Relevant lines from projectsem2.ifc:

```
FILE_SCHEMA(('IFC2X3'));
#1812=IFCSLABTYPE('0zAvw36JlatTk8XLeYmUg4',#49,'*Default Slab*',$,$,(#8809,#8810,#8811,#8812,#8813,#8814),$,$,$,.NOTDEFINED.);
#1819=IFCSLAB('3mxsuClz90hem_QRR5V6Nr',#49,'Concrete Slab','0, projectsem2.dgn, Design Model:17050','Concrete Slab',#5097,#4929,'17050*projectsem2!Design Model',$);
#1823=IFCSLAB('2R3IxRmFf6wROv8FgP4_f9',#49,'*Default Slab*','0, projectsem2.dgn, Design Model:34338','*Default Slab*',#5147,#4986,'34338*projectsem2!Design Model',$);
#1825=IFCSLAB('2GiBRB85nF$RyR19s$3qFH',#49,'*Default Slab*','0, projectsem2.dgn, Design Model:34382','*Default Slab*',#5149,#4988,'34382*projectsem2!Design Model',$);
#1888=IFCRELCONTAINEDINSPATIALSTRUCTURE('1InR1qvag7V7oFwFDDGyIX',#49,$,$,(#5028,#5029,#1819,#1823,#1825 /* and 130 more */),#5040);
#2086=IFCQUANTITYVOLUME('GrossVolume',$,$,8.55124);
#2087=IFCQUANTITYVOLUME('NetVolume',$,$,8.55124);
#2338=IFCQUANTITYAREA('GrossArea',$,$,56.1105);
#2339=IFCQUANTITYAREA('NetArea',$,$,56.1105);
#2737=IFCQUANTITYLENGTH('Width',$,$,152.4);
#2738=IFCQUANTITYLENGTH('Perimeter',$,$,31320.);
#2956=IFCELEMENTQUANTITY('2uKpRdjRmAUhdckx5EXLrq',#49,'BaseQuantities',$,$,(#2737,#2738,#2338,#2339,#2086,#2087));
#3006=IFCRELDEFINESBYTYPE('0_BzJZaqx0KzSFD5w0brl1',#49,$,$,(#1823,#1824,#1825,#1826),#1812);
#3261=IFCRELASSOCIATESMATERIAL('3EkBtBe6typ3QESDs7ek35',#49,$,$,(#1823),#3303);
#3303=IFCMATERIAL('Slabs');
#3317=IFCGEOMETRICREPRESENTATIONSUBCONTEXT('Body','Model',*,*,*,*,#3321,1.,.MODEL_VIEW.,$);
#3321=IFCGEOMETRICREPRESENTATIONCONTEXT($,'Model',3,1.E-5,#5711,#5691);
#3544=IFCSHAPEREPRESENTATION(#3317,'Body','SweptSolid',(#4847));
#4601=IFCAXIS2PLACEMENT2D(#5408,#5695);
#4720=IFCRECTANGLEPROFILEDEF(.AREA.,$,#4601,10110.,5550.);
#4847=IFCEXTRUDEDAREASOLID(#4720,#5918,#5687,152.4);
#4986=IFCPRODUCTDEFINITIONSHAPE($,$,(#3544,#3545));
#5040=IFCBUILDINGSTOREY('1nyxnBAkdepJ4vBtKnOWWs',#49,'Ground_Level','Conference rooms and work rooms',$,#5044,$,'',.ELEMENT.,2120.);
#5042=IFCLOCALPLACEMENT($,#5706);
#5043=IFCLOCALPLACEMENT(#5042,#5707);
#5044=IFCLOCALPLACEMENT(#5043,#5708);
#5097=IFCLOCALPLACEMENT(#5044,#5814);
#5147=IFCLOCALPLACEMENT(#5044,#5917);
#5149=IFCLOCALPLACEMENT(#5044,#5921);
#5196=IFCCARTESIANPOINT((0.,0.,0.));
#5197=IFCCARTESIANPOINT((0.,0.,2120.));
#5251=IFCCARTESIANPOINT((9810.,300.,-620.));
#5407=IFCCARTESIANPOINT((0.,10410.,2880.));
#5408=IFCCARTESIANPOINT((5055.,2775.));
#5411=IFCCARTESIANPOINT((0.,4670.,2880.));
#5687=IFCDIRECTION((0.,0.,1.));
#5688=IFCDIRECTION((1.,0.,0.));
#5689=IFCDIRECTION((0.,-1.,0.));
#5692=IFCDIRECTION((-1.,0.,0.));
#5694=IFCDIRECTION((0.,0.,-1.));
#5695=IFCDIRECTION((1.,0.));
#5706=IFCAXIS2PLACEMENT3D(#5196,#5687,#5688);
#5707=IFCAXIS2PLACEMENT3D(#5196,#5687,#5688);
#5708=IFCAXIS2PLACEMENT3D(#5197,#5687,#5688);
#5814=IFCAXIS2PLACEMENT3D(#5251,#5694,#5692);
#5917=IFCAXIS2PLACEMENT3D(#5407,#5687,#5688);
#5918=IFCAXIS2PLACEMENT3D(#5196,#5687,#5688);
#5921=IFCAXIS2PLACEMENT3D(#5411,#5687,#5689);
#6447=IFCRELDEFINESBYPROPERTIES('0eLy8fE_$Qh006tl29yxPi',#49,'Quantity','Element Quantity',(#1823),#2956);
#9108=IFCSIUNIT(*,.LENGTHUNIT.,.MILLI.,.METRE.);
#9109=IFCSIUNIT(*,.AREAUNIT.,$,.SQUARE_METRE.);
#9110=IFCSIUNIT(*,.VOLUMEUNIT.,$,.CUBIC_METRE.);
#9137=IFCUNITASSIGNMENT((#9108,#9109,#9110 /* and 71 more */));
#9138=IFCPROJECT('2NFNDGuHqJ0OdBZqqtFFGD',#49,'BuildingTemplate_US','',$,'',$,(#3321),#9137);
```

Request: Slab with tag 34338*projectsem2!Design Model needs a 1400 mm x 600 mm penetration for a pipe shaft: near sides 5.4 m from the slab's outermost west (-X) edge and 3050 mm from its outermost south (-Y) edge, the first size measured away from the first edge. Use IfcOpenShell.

```python
import numpy as np
import ifcopenshell
import ifcopenshell.api.feature
import ifcopenshell.api.geometry
import ifcopenshell.api.pset
import ifcopenshell.api.root
import ifcopenshell.geom
import ifcopenshell.util.element
import ifcopenshell.util.placement
import ifcopenshell.util.representation
import ifcopenshell.util.shape
import ifcopenshell.util.unit

model = ifcopenshell.open("projectsem2.ifc")
unit_scale = ifcopenshell.util.unit.calculate_unit_scale(model)
area_scale = ifcopenshell.util.unit.calculate_unit_scale(model, "AREAUNIT")
volume_scale = ifcopenshell.util.unit.calculate_unit_scale(model, "VOLUMEUNIT")
settings = ifcopenshell.geom.settings()


def volume(element):
    """Net volume in cubic metres, openings subtracted."""
    shape = ifcopenshell.geom.create_shape(settings, element)
    return ifcopenshell.util.shape.get_volume(shape.geometry)


slab = model.by_id(1823)
before = volume(slab)

# Extent in the slab's own axes, in metres. The edges named are its -X and -Y sides.
slab_shape = ifcopenshell.geom.create_shape(settings, slab)
vertices = ifcopenshell.util.shape.get_vertices(slab_shape.geometry)
x_min, y_min, bottom = vertices.min(axis=0)
top = vertices[:, 2].max()

opening = ifcopenshell.api.root.create_entity(model, ifc_class="IfcOpeningElement", name="Pipe shaft opening")
context = ifcopenshell.util.representation.get_context(model, "Model", "Body", "MODEL_VIEW")
width, depth = 1.4, 0.6
outline = [(0.0, 0.0), (width, 0.0), (width, depth), (0.0, depth), (0.0, 0.0)]
# Overshoot both faces by 50 mm so the cut is clean.
shape = ifcopenshell.api.geometry.add_slab_representation(
    model, context=context, depth=top - bottom + 0.1, polyline=outline
)
ifcopenshell.api.geometry.assign_representation(model, product=opening, representation=shape)

matrix = ifcopenshell.util.placement.get_local_placement(slab.ObjectPlacement)
matrix[:, 3] = matrix @ np.append(np.array([x_min + 5.4, y_min + 3.05, bottom - 0.05]) / unit_scale, 1.0)
ifcopenshell.api.geometry.edit_object_placement(model, product=opening, matrix=matrix, is_si=False)
ifcopenshell.api.feature.add_feature(model, feature=opening, element=slab)

after = volume(slab)

# Update the slab's stored quantities.
qto = model.by_id(ifcopenshell.util.element.get_pset(slab, "BaseQuantities", should_inherit=False)["id"])
ifcopenshell.api.pset.edit_qto(model, qto=qto, properties={
    "NetArea": after / (top - bottom) / area_scale,
    "NetVolume": after / volume_scale,
})

print(f"slab volume {before:.3f} -> {after:.3f} m3")

model.write("projectsem2_v2.ifc")
```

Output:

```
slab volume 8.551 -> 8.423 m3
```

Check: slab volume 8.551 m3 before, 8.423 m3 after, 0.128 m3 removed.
